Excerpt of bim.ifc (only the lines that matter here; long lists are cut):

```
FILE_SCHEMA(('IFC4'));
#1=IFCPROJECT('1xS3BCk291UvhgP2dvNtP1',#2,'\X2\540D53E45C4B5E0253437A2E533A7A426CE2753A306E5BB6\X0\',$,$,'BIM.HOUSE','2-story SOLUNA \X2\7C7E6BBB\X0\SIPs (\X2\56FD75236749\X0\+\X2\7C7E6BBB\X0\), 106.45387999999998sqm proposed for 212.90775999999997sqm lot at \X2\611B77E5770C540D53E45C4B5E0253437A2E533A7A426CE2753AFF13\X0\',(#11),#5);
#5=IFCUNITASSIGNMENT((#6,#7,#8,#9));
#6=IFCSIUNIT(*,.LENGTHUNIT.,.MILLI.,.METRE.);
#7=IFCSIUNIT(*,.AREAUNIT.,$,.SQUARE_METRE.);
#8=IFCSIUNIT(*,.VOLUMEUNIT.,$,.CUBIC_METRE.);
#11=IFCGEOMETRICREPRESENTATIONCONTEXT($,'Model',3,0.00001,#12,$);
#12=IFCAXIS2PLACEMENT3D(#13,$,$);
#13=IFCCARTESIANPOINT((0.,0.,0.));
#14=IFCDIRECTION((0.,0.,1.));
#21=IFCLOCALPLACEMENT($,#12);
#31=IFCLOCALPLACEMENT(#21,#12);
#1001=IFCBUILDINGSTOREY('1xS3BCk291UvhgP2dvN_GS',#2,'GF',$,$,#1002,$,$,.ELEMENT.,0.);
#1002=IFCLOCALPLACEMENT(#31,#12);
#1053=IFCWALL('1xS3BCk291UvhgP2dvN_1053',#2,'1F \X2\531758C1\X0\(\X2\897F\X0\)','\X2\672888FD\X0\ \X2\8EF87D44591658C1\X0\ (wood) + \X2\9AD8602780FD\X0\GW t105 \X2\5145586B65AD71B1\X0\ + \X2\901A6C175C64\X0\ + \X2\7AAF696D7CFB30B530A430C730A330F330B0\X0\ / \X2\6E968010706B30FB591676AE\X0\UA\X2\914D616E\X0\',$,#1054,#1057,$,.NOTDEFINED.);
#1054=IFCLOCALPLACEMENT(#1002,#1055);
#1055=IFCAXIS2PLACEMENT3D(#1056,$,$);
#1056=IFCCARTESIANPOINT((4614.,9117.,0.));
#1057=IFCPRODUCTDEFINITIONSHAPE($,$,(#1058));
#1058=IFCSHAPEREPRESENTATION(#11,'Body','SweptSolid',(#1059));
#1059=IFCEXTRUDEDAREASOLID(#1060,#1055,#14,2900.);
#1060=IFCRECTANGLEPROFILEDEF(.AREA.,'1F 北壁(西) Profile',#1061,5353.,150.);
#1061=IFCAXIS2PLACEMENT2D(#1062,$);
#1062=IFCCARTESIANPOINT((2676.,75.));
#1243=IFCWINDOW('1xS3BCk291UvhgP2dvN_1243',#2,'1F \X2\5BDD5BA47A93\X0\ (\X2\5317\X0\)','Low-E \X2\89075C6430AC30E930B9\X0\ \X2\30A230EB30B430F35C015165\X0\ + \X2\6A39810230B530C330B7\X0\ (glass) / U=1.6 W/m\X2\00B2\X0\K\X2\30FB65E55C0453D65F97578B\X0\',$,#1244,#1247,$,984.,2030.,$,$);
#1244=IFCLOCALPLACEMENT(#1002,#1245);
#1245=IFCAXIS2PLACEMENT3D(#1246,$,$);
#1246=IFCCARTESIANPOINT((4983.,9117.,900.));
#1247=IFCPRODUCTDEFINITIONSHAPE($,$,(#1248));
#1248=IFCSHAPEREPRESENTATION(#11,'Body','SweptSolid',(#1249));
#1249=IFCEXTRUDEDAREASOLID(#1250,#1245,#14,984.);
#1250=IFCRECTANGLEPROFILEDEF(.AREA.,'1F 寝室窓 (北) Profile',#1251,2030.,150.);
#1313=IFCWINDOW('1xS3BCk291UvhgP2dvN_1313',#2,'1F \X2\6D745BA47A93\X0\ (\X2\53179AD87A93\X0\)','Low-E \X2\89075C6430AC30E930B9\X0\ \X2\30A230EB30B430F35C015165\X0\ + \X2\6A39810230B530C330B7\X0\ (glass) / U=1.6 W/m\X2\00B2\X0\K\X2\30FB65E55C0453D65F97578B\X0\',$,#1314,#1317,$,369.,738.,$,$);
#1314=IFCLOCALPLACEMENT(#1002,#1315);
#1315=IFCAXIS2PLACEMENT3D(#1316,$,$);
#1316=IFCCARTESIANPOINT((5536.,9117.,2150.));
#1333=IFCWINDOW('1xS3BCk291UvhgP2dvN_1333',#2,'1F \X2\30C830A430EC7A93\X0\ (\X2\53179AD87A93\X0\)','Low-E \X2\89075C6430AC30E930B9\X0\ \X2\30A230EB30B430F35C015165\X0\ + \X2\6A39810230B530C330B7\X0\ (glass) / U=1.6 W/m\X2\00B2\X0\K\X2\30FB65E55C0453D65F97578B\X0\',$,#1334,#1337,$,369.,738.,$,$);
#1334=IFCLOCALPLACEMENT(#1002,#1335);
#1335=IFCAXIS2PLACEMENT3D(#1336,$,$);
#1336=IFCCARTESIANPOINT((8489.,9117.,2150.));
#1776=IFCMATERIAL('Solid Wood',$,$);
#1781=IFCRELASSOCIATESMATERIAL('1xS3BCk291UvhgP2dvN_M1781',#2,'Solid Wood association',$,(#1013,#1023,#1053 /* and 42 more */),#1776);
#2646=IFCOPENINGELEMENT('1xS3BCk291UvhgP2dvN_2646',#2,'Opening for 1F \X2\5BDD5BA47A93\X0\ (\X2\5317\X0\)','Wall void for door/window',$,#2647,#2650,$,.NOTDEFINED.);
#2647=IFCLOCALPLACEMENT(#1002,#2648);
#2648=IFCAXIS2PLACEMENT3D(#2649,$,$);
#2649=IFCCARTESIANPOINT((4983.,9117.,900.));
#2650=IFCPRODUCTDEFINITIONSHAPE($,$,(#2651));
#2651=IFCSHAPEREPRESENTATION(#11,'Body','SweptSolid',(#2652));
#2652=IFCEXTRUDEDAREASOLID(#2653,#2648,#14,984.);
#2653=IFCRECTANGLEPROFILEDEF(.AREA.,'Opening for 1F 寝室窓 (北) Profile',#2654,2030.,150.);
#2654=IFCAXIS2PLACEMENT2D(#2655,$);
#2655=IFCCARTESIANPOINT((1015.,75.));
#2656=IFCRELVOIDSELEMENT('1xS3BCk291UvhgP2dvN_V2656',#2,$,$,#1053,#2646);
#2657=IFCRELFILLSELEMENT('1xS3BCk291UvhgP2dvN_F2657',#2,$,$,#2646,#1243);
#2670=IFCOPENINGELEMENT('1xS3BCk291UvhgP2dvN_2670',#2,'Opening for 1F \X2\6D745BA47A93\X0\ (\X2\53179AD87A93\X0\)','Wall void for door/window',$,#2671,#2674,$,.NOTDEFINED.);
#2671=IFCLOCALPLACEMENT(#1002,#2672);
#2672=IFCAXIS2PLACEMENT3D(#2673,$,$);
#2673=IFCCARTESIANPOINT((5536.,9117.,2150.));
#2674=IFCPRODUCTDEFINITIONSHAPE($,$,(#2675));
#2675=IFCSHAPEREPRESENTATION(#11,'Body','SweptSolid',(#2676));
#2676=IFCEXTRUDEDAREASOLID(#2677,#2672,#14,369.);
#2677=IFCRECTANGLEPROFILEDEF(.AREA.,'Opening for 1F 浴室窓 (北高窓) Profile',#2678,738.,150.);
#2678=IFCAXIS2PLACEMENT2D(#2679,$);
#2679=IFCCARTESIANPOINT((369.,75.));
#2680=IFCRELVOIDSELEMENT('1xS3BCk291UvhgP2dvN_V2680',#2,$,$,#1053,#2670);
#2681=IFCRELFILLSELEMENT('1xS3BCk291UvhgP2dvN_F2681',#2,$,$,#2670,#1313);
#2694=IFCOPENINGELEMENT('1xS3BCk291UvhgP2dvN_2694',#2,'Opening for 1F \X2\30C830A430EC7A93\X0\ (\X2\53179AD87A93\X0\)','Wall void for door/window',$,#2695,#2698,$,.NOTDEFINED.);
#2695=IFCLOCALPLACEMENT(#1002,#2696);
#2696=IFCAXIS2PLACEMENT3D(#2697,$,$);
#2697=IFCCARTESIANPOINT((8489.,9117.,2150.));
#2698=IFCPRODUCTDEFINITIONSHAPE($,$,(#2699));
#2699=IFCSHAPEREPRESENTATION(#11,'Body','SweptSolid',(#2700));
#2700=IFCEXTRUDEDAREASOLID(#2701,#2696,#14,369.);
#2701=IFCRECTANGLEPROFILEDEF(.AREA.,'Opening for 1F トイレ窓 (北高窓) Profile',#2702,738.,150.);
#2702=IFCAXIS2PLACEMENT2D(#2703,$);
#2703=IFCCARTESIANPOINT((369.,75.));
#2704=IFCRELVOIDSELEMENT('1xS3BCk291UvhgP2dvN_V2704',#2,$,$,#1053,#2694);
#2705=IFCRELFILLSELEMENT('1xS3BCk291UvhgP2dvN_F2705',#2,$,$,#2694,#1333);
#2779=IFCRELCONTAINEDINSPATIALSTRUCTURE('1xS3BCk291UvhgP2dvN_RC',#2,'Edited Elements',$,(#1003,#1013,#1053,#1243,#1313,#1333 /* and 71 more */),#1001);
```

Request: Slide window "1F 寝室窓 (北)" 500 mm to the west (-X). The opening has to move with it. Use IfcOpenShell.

```python
import ifcopenshell
import ifcopenshell.api.geometry
import ifcopenshell.util.placement
import ifcopenshell.util.unit

model = ifcopenshell.open("bim.ifc")
unit_scale = ifcopenshell.util.unit.calculate_unit_scale(model)

window = model.by_id(1243)
opening = window.FillsVoids[0].RelatingOpeningElement
wall = opening.VoidsElements[0].RelatingBuildingElement

wall_matrix = ifcopenshell.util.placement.get_local_placement(wall.ObjectPlacement)
shift = wall_matrix[:3, 0] * -0.5 / unit_scale
before = ifcopenshell.util.placement.get_local_placement(window.ObjectPlacement)[:3, 3].copy()

# The window is not placed relative to its opening, so move both.
for product in (opening, window):
    matrix = ifcopenshell.util.placement.get_local_placement(product.ObjectPlacement)
    matrix[:3, 3] += shift
    ifcopenshell.api.geometry.edit_object_placement(model, product=product, matrix=matrix, is_si=False)

after = ifcopenshell.util.placement.get_local_placement(window.ObjectPlacement)[:3, 3]
print("window moved by", (after - before).round(3) + 0.0)

model.write("bim_v2.ifc")
```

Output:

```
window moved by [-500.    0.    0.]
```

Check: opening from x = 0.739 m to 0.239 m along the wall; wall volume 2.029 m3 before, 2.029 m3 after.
